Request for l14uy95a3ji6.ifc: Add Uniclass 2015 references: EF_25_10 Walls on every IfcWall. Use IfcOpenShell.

First a look at what the model holds.

```python
import ifcopenshell

model = ifcopenshell.open("l14uy95a3ji6.ifc")
print(model.schema)
print("classifications:", [c.Name for c in model.by_type("IfcClassification")])
for ifc_class in ("IfcDoor", "IfcRoof", "IfcStair", "IfcWall", "IfcWindow"):
    print(ifc_class, len(model.by_type(ifc_class)))
```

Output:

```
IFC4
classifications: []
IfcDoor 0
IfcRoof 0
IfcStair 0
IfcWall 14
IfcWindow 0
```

```python
import ifcopenshell
import ifcopenshell.api.classification

model = ifcopenshell.open("l14uy95a3ji6.ifc")

system = ifcopenshell.api.classification.add_classification(model, classification="Uniclass 2015")

codes = {
    "IfcWall": ("EF_25_10", "Walls"),
}
for ifc_class, (code, name) in codes.items():
    products = model.by_type(ifc_class)
    ifcopenshell.api.classification.add_reference(
        model, products=products, classification=system, identification=code, name=name
    )
    print(code, len(products))

model.write("l14uy95a3ji6_rev.ifc")
```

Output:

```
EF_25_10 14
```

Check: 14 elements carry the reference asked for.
